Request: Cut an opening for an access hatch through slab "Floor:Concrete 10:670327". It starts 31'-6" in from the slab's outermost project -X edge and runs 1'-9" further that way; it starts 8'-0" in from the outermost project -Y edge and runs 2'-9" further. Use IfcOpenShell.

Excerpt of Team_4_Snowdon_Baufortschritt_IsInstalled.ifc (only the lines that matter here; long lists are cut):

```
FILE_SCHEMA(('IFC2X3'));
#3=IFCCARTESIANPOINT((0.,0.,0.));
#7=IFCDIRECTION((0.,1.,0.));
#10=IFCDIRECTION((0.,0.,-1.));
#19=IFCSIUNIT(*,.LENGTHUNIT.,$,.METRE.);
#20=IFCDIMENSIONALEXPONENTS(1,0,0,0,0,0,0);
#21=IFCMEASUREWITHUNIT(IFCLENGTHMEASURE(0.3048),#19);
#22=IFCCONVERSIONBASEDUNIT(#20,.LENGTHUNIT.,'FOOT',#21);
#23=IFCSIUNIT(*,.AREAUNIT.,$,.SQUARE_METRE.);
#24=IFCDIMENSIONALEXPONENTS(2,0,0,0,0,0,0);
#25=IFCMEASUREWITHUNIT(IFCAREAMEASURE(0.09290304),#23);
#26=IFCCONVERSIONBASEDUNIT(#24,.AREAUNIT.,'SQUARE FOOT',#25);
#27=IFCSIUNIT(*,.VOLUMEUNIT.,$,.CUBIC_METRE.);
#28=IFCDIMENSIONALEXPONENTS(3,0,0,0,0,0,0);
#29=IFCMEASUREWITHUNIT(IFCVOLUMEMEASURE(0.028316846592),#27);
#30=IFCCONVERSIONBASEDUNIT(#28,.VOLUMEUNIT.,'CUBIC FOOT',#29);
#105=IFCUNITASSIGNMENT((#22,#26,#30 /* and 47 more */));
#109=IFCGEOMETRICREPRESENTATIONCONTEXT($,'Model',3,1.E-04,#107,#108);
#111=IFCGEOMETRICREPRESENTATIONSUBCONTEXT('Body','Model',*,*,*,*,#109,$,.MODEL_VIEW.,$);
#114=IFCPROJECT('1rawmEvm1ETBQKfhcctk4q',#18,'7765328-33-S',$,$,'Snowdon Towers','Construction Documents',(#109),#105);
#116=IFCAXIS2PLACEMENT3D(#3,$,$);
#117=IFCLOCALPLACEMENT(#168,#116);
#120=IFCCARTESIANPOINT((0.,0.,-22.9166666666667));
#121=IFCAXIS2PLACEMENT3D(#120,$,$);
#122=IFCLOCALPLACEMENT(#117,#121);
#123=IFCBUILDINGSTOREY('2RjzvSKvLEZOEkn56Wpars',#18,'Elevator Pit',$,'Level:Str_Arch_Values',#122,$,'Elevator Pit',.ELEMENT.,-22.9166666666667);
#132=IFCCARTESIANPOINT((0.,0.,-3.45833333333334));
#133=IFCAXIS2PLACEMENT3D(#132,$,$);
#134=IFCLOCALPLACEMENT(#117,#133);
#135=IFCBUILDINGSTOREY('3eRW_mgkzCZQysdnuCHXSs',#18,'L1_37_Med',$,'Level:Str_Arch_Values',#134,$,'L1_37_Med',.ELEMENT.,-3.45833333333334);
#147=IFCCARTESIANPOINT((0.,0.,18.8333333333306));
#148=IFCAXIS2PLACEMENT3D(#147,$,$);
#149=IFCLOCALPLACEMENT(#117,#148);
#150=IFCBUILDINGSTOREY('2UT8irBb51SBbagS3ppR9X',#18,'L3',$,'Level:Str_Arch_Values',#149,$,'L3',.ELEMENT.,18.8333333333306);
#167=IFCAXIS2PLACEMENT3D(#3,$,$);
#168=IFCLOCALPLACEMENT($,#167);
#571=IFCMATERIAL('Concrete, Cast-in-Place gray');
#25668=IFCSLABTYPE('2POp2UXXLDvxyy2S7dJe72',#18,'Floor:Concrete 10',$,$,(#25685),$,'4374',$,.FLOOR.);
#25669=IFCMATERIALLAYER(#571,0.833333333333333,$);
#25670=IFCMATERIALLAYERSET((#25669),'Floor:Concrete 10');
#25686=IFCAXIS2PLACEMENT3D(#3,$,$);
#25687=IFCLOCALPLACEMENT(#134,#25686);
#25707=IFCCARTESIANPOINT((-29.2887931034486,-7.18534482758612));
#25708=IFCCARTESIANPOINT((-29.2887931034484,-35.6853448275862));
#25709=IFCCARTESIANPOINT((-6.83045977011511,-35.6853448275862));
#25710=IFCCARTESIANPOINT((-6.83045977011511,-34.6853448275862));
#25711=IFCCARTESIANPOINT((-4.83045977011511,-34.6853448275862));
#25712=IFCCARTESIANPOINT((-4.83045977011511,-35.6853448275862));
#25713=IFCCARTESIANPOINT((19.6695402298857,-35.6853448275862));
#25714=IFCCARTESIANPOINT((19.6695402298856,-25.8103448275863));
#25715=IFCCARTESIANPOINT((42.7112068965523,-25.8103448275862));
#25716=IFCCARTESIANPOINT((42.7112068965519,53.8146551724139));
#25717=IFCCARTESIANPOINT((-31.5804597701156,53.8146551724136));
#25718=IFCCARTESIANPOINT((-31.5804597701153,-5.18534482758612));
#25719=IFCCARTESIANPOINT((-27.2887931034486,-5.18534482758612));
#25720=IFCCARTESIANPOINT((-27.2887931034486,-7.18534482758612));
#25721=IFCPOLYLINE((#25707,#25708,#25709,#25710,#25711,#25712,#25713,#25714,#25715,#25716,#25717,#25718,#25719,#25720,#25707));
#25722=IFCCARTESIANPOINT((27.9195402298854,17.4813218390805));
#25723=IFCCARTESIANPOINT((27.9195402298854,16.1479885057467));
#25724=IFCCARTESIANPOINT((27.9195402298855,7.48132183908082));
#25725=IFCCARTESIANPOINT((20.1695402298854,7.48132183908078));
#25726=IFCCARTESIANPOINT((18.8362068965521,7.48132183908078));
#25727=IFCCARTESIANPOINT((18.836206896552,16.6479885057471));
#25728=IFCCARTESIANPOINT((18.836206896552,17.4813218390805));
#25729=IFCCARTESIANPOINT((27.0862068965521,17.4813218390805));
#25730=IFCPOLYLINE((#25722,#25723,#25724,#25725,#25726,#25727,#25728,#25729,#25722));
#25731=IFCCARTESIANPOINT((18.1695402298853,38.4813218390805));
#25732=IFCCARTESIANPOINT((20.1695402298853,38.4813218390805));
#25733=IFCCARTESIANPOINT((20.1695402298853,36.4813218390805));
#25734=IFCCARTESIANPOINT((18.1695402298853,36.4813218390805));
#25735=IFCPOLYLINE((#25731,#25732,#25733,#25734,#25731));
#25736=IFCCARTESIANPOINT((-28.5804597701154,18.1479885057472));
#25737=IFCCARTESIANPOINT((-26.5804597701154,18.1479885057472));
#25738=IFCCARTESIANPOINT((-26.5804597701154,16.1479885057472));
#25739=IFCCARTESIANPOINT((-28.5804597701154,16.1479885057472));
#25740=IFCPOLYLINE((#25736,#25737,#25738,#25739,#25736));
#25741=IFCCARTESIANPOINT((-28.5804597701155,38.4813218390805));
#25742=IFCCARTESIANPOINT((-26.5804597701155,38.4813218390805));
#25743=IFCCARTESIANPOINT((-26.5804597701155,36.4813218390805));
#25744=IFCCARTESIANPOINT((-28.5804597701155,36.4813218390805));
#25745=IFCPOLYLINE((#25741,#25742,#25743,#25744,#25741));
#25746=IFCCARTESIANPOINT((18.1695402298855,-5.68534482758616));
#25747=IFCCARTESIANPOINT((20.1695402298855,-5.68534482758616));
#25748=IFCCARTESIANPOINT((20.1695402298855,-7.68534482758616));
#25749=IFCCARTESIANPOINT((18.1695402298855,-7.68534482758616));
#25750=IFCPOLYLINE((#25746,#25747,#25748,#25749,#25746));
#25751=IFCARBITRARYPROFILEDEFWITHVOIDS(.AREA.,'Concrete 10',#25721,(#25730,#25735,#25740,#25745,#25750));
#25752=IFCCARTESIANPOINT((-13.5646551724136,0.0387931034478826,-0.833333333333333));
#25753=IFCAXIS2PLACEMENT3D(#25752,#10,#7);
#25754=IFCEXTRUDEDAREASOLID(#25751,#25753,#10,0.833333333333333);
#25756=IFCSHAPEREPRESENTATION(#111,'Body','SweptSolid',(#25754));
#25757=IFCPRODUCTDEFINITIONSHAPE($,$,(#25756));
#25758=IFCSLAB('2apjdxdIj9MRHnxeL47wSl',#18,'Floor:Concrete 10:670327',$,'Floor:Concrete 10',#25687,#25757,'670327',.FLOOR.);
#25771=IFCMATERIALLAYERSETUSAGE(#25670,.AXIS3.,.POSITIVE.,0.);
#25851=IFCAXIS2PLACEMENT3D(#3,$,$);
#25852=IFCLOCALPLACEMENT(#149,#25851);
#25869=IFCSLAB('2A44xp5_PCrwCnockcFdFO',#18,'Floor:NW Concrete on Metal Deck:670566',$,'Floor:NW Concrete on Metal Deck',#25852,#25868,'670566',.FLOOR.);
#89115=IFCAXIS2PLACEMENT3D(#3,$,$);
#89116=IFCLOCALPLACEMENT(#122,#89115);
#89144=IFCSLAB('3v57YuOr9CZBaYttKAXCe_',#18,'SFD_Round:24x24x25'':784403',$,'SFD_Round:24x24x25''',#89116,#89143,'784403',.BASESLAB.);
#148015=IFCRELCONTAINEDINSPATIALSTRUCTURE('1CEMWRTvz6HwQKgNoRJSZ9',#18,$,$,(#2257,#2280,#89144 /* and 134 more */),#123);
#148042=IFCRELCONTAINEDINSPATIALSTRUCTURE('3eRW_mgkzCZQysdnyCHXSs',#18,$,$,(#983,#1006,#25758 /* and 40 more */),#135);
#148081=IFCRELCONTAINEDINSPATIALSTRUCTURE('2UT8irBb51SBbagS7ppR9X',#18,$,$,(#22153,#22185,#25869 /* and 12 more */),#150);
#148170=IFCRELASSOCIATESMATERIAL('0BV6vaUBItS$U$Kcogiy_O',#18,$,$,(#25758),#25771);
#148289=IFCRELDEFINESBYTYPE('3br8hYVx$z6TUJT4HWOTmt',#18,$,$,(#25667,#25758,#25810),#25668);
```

```python
import numpy as np
import ifcopenshell
import ifcopenshell.api.feature
import ifcopenshell.api.geometry
import ifcopenshell.api.root
import ifcopenshell.geom
import ifcopenshell.util.placement
import ifcopenshell.util.representation
import ifcopenshell.util.shape
import ifcopenshell.util.unit

model = ifcopenshell.open("Team_4_Snowdon_Baufortschritt_IsInstalled.ifc")
unit_scale = ifcopenshell.util.unit.calculate_unit_scale(model)
settings = ifcopenshell.geom.settings()


def volume(element):
    """Net volume in cubic metres, openings subtracted."""
    shape = ifcopenshell.geom.create_shape(settings, element)
    return ifcopenshell.util.shape.get_volume(shape.geometry)


slab = model.by_guid("2apjdxdIj9MRHnxeL47wSl")
before = volume(slab)

# Extent in the slab's own axes, in metres. The edges named are its -X and -Y sides.
slab_shape = ifcopenshell.geom.create_shape(settings, slab)
vertices = ifcopenshell.util.shape.get_vertices(slab_shape.geometry)
x_min, y_min, bottom = vertices.min(axis=0)
top = vertices[:, 2].max()

opening = ifcopenshell.api.root.create_entity(model, ifc_class="IfcOpeningElement", name="Access hatch opening")
context = ifcopenshell.util.representation.get_context(model, "Model", "Body", "MODEL_VIEW")
width, depth = 0.5334, 0.8382
outline = [(0.0, 0.0), (width, 0.0), (width, depth), (0.0, depth), (0.0, 0.0)]
# Overshoot both faces by 50 mm so the cut is clean.
shape = ifcopenshell.api.geometry.add_slab_representation(
    model, context=context, depth=top - bottom + 0.1, polyline=outline
)
ifcopenshell.api.geometry.assign_representation(model, product=opening, representation=shape)

matrix = ifcopenshell.util.placement.get_local_placement(slab.ObjectPlacement)
matrix[:, 3] = matrix @ np.append(np.array([x_min + 9.6012, y_min + 2.4384, bottom - 0.05]) / unit_scale, 1.0)
ifcopenshell.api.geometry.edit_object_placement(model, product=opening, matrix=matrix, is_si=False)
ifcopenshell.api.feature.add_feature(model, feature=opening, element=slab)

after = volume(slab)

print(f"slab volume {before:.3f} -> {after:.3f} m3")

model.write("Team_4_Snowdon_Baufortschritt_IsInstalled_edited.ifc")
```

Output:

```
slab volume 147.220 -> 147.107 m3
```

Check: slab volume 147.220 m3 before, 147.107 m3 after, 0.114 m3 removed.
